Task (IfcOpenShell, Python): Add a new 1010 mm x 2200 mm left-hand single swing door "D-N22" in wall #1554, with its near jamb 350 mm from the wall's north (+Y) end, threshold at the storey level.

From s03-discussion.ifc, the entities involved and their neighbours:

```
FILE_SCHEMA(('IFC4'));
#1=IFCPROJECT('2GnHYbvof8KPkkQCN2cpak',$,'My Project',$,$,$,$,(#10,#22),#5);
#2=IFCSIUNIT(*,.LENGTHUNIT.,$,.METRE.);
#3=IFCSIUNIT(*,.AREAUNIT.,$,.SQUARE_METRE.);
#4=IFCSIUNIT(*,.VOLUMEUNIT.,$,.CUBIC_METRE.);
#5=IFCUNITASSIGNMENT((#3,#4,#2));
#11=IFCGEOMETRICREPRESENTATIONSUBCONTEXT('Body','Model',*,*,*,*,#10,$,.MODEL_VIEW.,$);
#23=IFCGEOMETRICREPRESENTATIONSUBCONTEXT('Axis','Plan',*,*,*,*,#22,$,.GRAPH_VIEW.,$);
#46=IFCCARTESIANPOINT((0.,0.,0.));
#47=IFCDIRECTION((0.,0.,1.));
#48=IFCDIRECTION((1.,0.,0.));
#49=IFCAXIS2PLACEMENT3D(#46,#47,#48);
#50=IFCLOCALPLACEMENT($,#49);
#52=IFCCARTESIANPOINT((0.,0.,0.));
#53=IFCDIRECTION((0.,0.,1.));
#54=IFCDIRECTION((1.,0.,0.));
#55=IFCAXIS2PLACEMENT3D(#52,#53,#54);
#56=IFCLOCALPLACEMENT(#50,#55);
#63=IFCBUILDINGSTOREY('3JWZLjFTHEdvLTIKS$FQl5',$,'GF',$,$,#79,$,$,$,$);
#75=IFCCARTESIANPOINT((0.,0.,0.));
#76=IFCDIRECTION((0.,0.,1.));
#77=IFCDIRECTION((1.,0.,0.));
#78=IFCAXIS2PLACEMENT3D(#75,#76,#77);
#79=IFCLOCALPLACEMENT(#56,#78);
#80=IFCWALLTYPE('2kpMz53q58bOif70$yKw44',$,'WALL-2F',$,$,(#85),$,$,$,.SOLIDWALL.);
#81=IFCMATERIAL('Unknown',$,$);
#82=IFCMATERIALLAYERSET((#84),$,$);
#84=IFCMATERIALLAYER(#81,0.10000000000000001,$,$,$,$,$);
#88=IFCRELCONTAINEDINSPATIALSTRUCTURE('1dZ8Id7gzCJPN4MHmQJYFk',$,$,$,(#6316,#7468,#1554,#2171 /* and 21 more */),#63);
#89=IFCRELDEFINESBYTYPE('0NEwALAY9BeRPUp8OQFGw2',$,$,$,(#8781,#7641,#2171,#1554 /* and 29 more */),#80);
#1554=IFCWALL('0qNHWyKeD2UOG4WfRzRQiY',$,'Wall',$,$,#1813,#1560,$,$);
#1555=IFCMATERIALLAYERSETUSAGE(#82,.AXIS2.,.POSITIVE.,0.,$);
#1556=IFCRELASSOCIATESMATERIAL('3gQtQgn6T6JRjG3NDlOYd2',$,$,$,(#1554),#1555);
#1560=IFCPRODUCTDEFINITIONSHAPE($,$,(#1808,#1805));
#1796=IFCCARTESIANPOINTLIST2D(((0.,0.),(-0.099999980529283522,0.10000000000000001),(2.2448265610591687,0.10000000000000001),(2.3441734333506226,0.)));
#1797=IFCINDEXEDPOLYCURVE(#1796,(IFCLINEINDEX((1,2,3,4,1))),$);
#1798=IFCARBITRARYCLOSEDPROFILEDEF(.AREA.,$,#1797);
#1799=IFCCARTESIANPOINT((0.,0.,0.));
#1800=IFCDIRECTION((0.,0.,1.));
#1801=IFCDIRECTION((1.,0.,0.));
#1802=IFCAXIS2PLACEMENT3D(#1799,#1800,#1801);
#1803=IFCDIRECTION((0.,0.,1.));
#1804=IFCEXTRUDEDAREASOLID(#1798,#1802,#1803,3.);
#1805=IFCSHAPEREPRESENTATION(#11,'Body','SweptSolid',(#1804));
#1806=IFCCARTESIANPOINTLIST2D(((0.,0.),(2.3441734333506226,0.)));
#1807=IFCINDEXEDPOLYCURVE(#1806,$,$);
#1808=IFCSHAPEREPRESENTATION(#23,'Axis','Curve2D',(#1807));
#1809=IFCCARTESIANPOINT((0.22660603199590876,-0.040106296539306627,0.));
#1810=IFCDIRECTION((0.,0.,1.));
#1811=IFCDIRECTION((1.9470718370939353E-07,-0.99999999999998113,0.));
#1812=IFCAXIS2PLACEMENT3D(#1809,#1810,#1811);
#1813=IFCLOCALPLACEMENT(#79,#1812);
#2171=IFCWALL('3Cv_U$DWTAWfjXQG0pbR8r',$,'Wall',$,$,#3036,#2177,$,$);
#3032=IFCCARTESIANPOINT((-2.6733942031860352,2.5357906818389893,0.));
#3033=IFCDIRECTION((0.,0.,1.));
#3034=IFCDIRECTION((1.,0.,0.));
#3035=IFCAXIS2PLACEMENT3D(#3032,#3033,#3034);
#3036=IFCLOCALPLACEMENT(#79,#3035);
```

```python
import numpy as np
import ifcopenshell
import ifcopenshell.api.feature
import ifcopenshell.api.geometry
import ifcopenshell.api.root
import ifcopenshell.api.spatial
import ifcopenshell.geom
import ifcopenshell.util.element
import ifcopenshell.util.placement
import ifcopenshell.util.representation
import ifcopenshell.util.shape
import ifcopenshell.util.unit

model = ifcopenshell.open("s03-discussion.ifc")
unit_scale = ifcopenshell.util.unit.calculate_unit_scale(model)
settings = ifcopenshell.geom.settings()


def volume(element):
    """Net volume in cubic metres, openings subtracted."""
    shape = ifcopenshell.geom.create_shape(settings, element)
    return ifcopenshell.util.shape.get_volume(shape.geometry)


wall = model.by_id(1554)
storey = ifcopenshell.util.element.get_container(wall, ifc_class="IfcBuildingStorey")
context = ifcopenshell.util.representation.get_context(model, "Model", "Body", "MODEL_VIEW")
before = volume(wall)

width, height, from_end, sill = 1.01, 2.2, 0.35, 0.0  # metres

# The wall runs along its own X axis, and the end named is its -X end.
wall_shape = ifcopenshell.geom.create_shape(settings, wall)
x, y, z = ifcopenshell.util.shape.get_vertices(wall_shape.geometry).T
start = x.min() + from_end
face, thickness = float(y.min()), float(y.max() - y.min())
wall_matrix = ifcopenshell.util.placement.get_local_placement(wall.ObjectPlacement)
level = ifcopenshell.util.placement.get_local_placement(storey.ObjectPlacement)[2, 3]


def in_wall(x, y):
    """Placement at x, y metres in the wall's axes, at sill height."""
    matrix = wall_matrix.copy()
    matrix[:, 3] = wall_matrix @ np.array([x / unit_scale, y / unit_scale, 0.0, 1.0])
    matrix[2, 3] = level + sill / unit_scale
    return matrix


# Opening: a box that overshoots both wall faces by 50 mm.
opening = ifcopenshell.api.root.create_entity(model, ifc_class="IfcOpeningElement", predefined_type="OPENING")
box = ifcopenshell.api.geometry.add_wall_representation(
    model, context=context, length=width, height=height, thickness=thickness + 0.1
)
ifcopenshell.api.geometry.assign_representation(model, product=opening, representation=box)
ifcopenshell.api.geometry.edit_object_placement(model, product=opening, matrix=in_wall(start, face - 0.05), is_si=False)
ifcopenshell.api.feature.add_feature(model, feature=opening, element=wall)

door = ifcopenshell.api.root.create_entity(model, ifc_class="IfcDoor", name="D-N22", predefined_type="DOOR")
door.OverallWidth, door.OverallHeight = width / unit_scale, height / unit_scale
door.OperationType = "SINGLE_SWING_LEFT"
body = ifcopenshell.api.geometry.add_door_representation(
    model,
    context=context,
    overall_width=door.OverallWidth,
    overall_height=door.OverallHeight,
    operation_type="SINGLE_SWING_LEFT",
    lining_properties={"LiningDepth": thickness / unit_scale, "ThresholdDepth": thickness / unit_scale},
)
ifcopenshell.api.geometry.assign_representation(model, product=door, representation=body)
ifcopenshell.api.spatial.assign_container(model, products=[door], relating_structure=storey)
ifcopenshell.api.feature.add_filling(model, opening=opening, element=door)

# The lining spans the wall, so the door starts at the wall face.
ifcopenshell.api.geometry.edit_object_placement(model, product=door, matrix=in_wall(start, face), is_si=False)

after = volume(wall)

print(f"wall volume {before:.3f} -> {after:.3f} m3")

model.write("s03-discussion_edited.ifc")
```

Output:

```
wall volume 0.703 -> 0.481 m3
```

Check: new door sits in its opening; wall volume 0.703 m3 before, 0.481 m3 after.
